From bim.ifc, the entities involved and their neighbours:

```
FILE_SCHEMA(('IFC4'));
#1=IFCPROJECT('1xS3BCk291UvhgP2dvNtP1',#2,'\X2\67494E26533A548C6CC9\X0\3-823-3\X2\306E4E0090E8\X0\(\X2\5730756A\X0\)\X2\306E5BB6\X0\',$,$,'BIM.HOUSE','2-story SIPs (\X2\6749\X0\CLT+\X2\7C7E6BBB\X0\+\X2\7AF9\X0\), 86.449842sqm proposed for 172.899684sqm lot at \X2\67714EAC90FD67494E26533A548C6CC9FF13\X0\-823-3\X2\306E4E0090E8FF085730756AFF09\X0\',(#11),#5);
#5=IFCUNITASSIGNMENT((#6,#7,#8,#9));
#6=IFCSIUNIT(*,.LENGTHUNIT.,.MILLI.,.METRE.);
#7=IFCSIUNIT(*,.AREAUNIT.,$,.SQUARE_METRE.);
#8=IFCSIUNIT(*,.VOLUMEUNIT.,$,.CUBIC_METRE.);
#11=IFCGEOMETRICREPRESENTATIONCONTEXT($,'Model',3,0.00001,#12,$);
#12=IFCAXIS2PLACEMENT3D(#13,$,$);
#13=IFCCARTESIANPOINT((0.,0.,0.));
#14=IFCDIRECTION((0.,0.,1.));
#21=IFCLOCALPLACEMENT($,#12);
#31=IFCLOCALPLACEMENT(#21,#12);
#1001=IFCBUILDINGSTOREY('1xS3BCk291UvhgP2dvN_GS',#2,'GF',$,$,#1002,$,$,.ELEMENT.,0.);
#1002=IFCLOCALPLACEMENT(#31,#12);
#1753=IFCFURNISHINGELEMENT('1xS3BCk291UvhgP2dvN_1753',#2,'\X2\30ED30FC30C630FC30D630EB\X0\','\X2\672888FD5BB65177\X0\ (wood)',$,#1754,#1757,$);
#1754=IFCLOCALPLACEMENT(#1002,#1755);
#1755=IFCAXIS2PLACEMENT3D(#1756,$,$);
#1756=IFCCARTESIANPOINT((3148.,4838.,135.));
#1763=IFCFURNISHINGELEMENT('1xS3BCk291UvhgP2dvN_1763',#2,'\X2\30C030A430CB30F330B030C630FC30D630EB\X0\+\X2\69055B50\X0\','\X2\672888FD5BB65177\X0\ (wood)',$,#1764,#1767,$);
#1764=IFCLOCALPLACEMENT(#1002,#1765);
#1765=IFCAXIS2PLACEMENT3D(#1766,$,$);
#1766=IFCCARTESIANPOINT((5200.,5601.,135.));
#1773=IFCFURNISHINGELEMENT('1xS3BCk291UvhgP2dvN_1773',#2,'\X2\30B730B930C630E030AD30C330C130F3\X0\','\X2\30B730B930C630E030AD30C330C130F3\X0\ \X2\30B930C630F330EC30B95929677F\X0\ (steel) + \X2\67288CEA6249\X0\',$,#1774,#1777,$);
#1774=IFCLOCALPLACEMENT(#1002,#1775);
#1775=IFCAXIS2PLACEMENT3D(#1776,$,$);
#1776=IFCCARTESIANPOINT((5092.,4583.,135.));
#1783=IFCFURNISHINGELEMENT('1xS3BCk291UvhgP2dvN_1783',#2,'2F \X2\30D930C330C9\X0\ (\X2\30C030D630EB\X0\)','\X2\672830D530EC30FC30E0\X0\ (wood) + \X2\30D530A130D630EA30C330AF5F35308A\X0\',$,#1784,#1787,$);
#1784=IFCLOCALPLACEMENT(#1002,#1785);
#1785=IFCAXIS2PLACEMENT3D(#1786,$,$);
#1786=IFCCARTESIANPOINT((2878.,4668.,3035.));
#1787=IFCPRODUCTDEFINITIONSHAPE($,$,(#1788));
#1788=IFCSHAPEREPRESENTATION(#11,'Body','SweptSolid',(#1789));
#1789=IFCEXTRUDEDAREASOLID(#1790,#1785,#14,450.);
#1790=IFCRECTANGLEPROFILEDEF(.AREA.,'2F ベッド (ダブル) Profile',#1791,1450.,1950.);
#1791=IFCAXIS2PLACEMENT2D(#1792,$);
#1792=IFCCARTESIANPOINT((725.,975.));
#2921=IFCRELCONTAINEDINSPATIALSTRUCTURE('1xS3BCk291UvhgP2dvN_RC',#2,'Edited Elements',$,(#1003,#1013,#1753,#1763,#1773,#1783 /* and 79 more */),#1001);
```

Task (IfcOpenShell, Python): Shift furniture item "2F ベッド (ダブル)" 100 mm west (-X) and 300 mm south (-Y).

```python
import ifcopenshell
import ifcopenshell.api.geometry
import ifcopenshell.util.placement

model = ifcopenshell.open("bim.ifc")

item = model.by_id(1783)
matrix = ifcopenshell.util.placement.get_local_placement(item.ObjectPlacement)
matrix[0, 3] -= 100.0
matrix[1, 3] -= 300.0
ifcopenshell.api.geometry.edit_object_placement(model, product=item, matrix=matrix, is_si=False)

print(ifcopenshell.util.placement.get_local_placement(item.ObjectPlacement).round(3) + 0.0)

model.write("bim-out.ifc")
```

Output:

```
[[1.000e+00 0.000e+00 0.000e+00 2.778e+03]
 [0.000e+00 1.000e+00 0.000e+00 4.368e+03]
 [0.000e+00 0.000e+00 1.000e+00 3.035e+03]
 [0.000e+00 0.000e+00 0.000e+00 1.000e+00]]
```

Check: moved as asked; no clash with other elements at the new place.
